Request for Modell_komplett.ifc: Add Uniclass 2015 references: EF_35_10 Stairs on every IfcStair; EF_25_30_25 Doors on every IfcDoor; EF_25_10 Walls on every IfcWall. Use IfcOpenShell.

First a look at what the model holds.

```python
import ifcopenshell

model = ifcopenshell.open("Modell_komplett.ifc")
print(model.schema)
print("classifications:", [c.Name for c in model.by_type("IfcClassification")])
for ifc_class in ("IfcDoor", "IfcRoof", "IfcStair", "IfcWall", "IfcWindow"):
    print(ifc_class, len(model.by_type(ifc_class)))
```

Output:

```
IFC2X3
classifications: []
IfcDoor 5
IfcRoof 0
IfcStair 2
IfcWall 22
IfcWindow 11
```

```python
import ifcopenshell
import ifcopenshell.api.classification

model = ifcopenshell.open("Modell_komplett.ifc")

# IFC2X3 requires Source and Edition and has no link from the project to the system.
system = model.create_entity("IfcClassification", Source="NBS", Edition="2015", Name="Uniclass 2015")

codes = {
    "IfcStair": ("EF_35_10", "Stairs"),
    "IfcDoor": ("EF_25_30_25", "Doors"),
    "IfcWall": ("EF_25_10", "Walls"),
}
for ifc_class, (code, name) in codes.items():
    products = model.by_type(ifc_class)
    ifcopenshell.api.classification.add_reference(
        model, products=products, classification=system, identification=code, name=name
    )
    print(code, len(products))

model.write("Modell_komplett_rev.ifc")
```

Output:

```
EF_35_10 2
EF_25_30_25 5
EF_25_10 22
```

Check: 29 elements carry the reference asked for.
